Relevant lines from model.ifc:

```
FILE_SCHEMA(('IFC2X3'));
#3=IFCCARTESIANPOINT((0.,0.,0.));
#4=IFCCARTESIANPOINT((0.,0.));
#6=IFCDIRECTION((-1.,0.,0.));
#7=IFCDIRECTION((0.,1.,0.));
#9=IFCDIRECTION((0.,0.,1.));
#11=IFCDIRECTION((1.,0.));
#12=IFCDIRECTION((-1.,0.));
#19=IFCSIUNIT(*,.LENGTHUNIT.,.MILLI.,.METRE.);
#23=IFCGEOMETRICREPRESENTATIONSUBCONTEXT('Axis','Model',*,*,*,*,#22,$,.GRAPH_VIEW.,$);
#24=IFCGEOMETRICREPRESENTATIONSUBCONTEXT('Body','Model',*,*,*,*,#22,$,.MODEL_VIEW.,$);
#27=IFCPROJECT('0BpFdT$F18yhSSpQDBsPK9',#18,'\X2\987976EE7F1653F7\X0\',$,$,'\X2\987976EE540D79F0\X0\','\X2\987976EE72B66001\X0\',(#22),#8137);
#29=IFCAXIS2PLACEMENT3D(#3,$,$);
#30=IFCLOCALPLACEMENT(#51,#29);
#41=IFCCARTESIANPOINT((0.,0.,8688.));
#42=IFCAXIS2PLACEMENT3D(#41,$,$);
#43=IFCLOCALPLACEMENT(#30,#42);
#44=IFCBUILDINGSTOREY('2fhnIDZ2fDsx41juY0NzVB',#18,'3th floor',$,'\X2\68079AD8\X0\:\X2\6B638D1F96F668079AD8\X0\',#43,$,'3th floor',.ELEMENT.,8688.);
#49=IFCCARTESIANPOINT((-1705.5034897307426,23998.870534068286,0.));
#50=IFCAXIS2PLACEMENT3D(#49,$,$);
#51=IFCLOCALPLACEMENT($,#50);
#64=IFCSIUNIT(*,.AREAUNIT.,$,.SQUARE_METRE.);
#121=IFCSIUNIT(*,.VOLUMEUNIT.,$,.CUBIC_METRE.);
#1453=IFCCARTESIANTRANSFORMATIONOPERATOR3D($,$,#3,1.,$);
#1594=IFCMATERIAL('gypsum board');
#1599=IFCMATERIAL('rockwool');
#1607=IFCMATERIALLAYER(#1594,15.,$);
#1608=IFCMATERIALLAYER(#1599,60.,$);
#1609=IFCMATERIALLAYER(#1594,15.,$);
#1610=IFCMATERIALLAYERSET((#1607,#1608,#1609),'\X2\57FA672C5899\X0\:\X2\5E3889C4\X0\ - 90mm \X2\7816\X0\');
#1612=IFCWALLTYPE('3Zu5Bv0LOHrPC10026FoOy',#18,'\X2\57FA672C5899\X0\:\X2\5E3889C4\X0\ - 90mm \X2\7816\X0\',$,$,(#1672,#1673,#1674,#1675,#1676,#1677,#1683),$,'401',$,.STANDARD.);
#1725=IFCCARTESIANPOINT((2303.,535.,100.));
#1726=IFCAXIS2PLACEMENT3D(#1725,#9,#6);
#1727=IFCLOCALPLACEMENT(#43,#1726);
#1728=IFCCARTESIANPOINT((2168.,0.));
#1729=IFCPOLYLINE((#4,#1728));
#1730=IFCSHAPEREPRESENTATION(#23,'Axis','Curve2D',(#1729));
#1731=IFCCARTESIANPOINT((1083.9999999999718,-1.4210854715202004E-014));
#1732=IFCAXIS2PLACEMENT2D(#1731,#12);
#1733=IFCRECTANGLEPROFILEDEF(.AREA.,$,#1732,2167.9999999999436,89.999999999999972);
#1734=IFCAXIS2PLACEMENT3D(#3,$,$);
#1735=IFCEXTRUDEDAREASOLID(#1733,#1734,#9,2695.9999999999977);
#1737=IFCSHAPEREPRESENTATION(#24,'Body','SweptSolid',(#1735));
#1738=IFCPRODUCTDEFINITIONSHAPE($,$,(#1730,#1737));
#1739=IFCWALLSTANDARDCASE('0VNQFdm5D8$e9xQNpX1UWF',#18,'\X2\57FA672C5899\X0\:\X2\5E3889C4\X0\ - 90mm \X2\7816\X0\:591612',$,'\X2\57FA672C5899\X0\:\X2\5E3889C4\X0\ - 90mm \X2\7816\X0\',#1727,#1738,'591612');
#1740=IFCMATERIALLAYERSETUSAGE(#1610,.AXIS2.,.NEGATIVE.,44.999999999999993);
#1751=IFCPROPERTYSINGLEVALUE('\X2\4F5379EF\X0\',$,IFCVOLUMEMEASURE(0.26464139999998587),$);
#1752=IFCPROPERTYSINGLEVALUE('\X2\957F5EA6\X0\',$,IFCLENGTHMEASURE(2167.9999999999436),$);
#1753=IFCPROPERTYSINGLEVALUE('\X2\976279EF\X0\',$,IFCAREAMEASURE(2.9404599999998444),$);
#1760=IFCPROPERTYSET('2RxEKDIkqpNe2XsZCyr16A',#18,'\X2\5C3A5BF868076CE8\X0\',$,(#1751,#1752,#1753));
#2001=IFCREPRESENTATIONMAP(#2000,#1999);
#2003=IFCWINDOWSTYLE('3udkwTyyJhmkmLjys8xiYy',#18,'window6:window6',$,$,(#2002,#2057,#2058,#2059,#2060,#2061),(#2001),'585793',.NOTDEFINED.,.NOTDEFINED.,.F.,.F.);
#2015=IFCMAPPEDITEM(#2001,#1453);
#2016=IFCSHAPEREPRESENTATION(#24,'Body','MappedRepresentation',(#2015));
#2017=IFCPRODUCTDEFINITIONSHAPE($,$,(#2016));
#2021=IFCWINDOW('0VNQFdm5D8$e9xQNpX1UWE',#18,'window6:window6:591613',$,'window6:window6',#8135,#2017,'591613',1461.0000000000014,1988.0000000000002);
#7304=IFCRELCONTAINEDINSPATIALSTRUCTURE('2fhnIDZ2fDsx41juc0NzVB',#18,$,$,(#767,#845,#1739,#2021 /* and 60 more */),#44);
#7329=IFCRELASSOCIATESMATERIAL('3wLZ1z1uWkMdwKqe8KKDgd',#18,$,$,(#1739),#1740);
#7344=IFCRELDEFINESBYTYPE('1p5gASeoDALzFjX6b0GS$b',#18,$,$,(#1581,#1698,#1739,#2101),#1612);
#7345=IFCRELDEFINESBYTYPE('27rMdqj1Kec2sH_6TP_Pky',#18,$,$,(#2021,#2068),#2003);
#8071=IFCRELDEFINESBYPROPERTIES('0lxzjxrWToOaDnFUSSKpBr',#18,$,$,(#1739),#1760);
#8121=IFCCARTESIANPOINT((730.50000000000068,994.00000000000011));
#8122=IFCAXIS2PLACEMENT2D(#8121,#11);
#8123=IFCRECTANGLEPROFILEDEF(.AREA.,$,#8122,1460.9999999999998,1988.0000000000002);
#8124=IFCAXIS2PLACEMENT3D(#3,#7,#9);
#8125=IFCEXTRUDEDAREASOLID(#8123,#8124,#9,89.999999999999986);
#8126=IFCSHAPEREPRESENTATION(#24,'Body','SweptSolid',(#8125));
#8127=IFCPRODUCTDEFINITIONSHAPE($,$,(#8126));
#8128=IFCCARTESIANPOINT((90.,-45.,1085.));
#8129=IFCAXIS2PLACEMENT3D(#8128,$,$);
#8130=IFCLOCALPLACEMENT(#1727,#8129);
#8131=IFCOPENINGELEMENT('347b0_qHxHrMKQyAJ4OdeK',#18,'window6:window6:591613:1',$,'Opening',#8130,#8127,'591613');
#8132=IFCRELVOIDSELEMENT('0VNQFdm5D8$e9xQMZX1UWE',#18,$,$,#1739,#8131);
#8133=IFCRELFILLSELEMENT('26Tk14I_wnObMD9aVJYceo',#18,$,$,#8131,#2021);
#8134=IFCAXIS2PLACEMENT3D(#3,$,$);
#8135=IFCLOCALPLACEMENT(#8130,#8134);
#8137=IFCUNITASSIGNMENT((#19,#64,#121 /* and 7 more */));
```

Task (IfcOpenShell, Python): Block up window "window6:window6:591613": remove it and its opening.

```python
import ifcopenshell
import ifcopenshell.api.feature
import ifcopenshell.api.pset
import ifcopenshell.api.root
import ifcopenshell.geom
import ifcopenshell.util.element
import ifcopenshell.util.shape
import ifcopenshell.util.unit

model = ifcopenshell.open("model.ifc")
area_scale = ifcopenshell.util.unit.calculate_unit_scale(model, "AREAUNIT")
volume_scale = ifcopenshell.util.unit.calculate_unit_scale(model, "VOLUMEUNIT")
settings = ifcopenshell.geom.settings()


def volume(element):
    """Net volume in cubic metres, openings subtracted."""
    shape = ifcopenshell.geom.create_shape(settings, element)
    return ifcopenshell.util.shape.get_volume(shape.geometry)


window = model.by_guid("0VNQFdm5D8$e9xQNpX1UWE")
opening = window.FillsVoids[0].RelatingOpeningElement
wall = opening.VoidsElements[0].RelatingBuildingElement
before = volume(wall)

ifcopenshell.api.root.remove_product(model, product=window)
ifcopenshell.api.feature.remove_feature(model, feature=opening)

after = volume(wall)
thickness = 0.09  # wall thickness in metres

# Update the wall's stored quantities.
pset = model.by_id(ifcopenshell.util.element.get_pset(wall, "尺寸标注", should_inherit=False)["id"])
ifcopenshell.api.pset.edit_pset(model, pset=pset, properties={
    "体积": model.create_entity("IfcVolumeMeasure", after / volume_scale),
    "面积": model.create_entity("IfcAreaMeasure", after / thickness / area_scale),
})

print(f"wall volume {before:.3f} -> {after:.3f} m3")

model.write("model_updated.ifc")
```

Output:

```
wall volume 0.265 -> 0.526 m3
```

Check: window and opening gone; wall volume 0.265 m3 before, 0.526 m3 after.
